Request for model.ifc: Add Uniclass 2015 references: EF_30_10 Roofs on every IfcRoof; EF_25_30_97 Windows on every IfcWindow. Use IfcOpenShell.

First a look at what the model holds.

```python
import ifcopenshell

model = ifcopenshell.open("model.ifc")
print(model.schema)
print("classifications:", [c.Name for c in model.by_type("IfcClassification")])
for ifc_class in ("IfcDoor", "IfcRoof", "IfcStair", "IfcWall", "IfcWindow"):
    print(ifc_class, len(model.by_type(ifc_class)))
```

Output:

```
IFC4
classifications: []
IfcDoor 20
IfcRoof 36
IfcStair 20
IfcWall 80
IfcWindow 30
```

```python
import ifcopenshell
import ifcopenshell.api.classification

model = ifcopenshell.open("model.ifc")

system = ifcopenshell.api.classification.add_classification(model, classification="Uniclass 2015")

codes = {
    "IfcRoof": ("EF_30_10", "Roofs"),
    "IfcWindow": ("EF_25_30_97", "Windows"),
}
for ifc_class, (code, name) in codes.items():
    products = model.by_type(ifc_class)
    ifcopenshell.api.classification.add_reference(
        model, products=products, classification=system, identification=code, name=name
    )
    print(code, len(products))

model.write("model_v2.ifc")
```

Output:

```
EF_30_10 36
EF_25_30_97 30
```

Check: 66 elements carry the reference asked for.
